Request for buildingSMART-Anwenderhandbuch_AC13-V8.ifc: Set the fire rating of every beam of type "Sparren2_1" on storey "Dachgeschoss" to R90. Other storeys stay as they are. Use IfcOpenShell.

First a look at what the model holds.

```python
import ifcopenshell
import ifcopenshell.util.element

model = ifcopenshell.open("buildingSMART-Anwenderhandbuch_AC13-V8.ifc")
print(model.schema)
storey = next(s for s in model.by_type("IfcBuildingStorey") if s.Name == "Dachgeschoss")
beams = [e for e in ifcopenshell.util.element.get_decomposition(storey) if e.is_a("IfcBeam")]
seen = {}
for e in beams:
    element_type = ifcopenshell.util.element.get_type(e)
    key = (element_type.Name if element_type != e and element_type else None, ifcopenshell.util.element.get_pset(e, "Pset_BeamCommon", "FireRating"))
    seen[key] = seen.get(key, 0) + 1
for (name, value), count in sorted(seen.items(), key=str):
    print(count, "x", name, "|", value)
```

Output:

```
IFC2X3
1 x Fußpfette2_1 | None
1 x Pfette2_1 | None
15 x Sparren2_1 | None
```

```python
import ifcopenshell
import ifcopenshell.api.pset
import ifcopenshell.util.element

model = ifcopenshell.open("buildingSMART-Anwenderhandbuch_AC13-V8.ifc")

storey = next(s for s in model.by_type("IfcBuildingStorey") if s.Name == "Dachgeschoss")
beams = [e for e in ifcopenshell.util.element.get_decomposition(storey) if e.is_a("IfcBeam")]

count = 0
for e in beams:
    element_type = ifcopenshell.util.element.get_type(e)
    if element_type in (None, e) or element_type.Name != "Sparren2_1":
        continue
    # add_pset returns the element's existing set when there is one.
    pset = ifcopenshell.api.pset.add_pset(model, product=e, name="Pset_BeamCommon")
    ifcopenshell.api.pset.edit_pset(model, pset=pset, properties={"FireRating": "R90"})
    count += 1

print(count, "beams updated")

model.write("buildingSMART-Anwenderhandbuch_AC13-V8_rev.ifc")
```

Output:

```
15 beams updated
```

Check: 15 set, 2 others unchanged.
